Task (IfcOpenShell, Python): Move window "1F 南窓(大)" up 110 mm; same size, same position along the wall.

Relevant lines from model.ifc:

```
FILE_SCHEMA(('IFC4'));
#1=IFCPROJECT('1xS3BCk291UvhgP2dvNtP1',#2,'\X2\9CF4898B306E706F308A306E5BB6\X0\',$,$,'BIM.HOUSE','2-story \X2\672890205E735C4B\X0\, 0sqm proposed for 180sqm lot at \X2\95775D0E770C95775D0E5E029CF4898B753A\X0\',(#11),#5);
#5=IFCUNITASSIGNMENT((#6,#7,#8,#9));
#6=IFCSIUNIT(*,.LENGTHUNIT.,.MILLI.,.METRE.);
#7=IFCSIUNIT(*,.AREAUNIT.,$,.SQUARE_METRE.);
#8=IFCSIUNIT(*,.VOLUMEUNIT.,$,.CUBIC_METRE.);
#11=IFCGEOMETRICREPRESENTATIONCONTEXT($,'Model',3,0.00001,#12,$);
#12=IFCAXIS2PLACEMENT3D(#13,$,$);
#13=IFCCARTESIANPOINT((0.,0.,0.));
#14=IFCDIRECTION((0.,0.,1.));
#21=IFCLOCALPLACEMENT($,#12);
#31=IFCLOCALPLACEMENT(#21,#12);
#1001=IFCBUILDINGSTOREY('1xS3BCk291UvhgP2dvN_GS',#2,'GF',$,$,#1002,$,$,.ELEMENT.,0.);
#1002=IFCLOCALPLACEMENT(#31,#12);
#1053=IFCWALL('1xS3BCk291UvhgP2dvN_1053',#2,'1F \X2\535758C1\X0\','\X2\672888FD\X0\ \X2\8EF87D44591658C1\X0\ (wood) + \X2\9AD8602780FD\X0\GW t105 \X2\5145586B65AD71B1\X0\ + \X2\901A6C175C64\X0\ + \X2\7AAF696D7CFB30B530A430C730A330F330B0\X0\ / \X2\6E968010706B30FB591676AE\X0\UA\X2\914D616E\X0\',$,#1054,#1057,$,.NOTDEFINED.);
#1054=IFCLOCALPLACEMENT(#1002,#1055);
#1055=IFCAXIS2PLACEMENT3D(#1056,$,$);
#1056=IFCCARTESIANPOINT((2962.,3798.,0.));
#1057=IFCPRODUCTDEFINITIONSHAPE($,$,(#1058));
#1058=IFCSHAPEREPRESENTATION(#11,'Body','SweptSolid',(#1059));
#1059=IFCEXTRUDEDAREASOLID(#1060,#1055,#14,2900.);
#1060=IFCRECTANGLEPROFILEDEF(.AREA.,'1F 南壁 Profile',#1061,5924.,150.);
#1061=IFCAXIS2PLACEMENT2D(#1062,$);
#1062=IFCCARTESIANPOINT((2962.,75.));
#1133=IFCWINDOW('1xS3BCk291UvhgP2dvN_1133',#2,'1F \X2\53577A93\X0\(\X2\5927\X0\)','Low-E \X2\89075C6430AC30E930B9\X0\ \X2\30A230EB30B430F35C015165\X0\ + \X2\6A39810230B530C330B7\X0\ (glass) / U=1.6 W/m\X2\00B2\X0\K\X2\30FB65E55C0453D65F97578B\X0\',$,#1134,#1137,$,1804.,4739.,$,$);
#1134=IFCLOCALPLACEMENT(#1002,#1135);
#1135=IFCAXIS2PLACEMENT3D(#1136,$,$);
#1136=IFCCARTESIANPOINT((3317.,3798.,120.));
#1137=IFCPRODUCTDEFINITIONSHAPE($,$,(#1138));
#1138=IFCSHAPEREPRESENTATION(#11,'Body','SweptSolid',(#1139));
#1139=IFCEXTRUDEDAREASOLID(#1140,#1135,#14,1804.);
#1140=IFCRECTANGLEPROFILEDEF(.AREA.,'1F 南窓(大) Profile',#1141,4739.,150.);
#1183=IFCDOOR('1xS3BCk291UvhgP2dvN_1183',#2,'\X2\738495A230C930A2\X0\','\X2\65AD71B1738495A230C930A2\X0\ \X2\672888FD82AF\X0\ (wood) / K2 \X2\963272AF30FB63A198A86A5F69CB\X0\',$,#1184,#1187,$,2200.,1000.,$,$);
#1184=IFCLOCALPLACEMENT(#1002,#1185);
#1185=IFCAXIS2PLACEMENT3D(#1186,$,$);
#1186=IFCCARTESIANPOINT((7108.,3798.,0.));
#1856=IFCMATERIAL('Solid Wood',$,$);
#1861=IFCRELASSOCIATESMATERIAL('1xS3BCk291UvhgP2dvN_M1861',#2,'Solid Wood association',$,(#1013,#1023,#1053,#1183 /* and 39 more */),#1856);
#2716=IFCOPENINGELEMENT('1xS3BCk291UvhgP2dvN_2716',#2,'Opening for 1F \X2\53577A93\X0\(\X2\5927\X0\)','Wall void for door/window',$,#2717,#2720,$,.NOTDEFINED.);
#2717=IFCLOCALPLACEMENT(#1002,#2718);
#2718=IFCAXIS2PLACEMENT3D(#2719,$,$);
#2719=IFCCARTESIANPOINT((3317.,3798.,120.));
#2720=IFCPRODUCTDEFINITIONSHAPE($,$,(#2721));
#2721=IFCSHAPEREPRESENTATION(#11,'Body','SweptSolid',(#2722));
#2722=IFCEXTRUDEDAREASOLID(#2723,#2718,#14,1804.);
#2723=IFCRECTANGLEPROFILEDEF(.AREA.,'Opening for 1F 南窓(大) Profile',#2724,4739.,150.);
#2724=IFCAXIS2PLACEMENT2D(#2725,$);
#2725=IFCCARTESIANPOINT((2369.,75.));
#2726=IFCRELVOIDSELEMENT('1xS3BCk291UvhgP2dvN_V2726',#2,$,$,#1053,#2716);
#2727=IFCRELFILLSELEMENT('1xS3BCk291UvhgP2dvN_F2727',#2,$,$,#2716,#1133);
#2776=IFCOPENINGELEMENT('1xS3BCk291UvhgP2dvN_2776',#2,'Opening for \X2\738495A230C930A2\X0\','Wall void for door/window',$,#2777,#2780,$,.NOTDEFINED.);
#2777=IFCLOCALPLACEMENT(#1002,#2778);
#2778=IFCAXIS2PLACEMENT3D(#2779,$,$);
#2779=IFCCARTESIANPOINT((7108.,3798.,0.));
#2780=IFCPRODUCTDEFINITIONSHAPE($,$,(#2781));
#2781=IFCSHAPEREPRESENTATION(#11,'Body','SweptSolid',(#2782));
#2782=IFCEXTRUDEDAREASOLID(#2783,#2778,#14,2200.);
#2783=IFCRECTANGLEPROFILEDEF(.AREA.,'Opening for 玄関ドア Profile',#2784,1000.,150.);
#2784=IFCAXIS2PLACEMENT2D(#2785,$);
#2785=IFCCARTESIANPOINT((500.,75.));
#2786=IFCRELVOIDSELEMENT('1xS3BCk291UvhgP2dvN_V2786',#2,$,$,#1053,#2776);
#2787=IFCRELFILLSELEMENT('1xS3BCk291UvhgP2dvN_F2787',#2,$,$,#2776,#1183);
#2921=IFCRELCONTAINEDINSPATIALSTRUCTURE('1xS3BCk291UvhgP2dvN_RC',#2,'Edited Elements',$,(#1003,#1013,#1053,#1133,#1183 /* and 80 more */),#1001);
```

```python
import numpy as np
import ifcopenshell
import ifcopenshell.api.geometry
import ifcopenshell.util.placement
import ifcopenshell.util.unit

model = ifcopenshell.open("model.ifc")
unit_scale = ifcopenshell.util.unit.calculate_unit_scale(model)

window = model.by_guid("1xS3BCk291UvhgP2dvN_1133")
opening = window.FillsVoids[0].RelatingOpeningElement
dz = 0.11 / unit_scale

shift = np.array([0.0, 0.0, dz])
# The window is not placed relative to its opening, so move both.
for product in (opening, window):
    matrix = ifcopenshell.util.placement.get_local_placement(product.ObjectPlacement)
    matrix[:3, 3] += shift
    ifcopenshell.api.geometry.edit_object_placement(model, product=product, matrix=matrix, is_si=False)

print(f"moved by {dz * unit_scale:+.3f} m")

model.write("model_v2.ifc")
```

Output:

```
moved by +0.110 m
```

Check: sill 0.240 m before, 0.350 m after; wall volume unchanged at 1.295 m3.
